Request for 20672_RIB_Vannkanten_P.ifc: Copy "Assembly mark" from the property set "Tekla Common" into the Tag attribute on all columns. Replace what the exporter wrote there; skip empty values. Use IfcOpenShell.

First a look at what the model holds.

```python
import ifcopenshell
import ifcopenshell.util.element

model = ifcopenshell.open("20672_RIB_Vannkanten_P.ifc")
print(model.schema)
columns = model.by_type("IfcColumn")
print(len(columns), "columns")
for e in columns[:8]:
    source = ifcopenshell.util.element.get_pset(e, "Tekla Common", "Assembly mark")
    target = e.Tag
    print(e.id(), repr(source), repr(target), sep=" | ")
```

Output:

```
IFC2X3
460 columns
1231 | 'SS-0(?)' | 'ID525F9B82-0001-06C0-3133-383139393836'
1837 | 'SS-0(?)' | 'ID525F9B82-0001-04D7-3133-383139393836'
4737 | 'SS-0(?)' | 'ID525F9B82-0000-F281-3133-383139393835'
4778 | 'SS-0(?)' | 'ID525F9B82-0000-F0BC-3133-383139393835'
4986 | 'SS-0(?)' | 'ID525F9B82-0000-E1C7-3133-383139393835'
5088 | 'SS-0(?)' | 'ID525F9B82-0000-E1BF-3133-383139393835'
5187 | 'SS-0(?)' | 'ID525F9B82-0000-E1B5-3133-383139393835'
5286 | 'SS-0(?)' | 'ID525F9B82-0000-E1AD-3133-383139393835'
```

```python
import ifcopenshell
import ifcopenshell.util.element

model = ifcopenshell.open("20672_RIB_Vannkanten_P.ifc")

count = 0
for e in model.by_type("IfcColumn"):
    value = ifcopenshell.util.element.get_pset(e, "Tekla Common", "Assembly mark")
    current = e.Tag
    if not value or not value.strip() or current == value:
        continue
    e.Tag = value
    count += 1

print(count, "columns updated")

model.write("20672_RIB_Vannkanten_P_rev.ifc")
```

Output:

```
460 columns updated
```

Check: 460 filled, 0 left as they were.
